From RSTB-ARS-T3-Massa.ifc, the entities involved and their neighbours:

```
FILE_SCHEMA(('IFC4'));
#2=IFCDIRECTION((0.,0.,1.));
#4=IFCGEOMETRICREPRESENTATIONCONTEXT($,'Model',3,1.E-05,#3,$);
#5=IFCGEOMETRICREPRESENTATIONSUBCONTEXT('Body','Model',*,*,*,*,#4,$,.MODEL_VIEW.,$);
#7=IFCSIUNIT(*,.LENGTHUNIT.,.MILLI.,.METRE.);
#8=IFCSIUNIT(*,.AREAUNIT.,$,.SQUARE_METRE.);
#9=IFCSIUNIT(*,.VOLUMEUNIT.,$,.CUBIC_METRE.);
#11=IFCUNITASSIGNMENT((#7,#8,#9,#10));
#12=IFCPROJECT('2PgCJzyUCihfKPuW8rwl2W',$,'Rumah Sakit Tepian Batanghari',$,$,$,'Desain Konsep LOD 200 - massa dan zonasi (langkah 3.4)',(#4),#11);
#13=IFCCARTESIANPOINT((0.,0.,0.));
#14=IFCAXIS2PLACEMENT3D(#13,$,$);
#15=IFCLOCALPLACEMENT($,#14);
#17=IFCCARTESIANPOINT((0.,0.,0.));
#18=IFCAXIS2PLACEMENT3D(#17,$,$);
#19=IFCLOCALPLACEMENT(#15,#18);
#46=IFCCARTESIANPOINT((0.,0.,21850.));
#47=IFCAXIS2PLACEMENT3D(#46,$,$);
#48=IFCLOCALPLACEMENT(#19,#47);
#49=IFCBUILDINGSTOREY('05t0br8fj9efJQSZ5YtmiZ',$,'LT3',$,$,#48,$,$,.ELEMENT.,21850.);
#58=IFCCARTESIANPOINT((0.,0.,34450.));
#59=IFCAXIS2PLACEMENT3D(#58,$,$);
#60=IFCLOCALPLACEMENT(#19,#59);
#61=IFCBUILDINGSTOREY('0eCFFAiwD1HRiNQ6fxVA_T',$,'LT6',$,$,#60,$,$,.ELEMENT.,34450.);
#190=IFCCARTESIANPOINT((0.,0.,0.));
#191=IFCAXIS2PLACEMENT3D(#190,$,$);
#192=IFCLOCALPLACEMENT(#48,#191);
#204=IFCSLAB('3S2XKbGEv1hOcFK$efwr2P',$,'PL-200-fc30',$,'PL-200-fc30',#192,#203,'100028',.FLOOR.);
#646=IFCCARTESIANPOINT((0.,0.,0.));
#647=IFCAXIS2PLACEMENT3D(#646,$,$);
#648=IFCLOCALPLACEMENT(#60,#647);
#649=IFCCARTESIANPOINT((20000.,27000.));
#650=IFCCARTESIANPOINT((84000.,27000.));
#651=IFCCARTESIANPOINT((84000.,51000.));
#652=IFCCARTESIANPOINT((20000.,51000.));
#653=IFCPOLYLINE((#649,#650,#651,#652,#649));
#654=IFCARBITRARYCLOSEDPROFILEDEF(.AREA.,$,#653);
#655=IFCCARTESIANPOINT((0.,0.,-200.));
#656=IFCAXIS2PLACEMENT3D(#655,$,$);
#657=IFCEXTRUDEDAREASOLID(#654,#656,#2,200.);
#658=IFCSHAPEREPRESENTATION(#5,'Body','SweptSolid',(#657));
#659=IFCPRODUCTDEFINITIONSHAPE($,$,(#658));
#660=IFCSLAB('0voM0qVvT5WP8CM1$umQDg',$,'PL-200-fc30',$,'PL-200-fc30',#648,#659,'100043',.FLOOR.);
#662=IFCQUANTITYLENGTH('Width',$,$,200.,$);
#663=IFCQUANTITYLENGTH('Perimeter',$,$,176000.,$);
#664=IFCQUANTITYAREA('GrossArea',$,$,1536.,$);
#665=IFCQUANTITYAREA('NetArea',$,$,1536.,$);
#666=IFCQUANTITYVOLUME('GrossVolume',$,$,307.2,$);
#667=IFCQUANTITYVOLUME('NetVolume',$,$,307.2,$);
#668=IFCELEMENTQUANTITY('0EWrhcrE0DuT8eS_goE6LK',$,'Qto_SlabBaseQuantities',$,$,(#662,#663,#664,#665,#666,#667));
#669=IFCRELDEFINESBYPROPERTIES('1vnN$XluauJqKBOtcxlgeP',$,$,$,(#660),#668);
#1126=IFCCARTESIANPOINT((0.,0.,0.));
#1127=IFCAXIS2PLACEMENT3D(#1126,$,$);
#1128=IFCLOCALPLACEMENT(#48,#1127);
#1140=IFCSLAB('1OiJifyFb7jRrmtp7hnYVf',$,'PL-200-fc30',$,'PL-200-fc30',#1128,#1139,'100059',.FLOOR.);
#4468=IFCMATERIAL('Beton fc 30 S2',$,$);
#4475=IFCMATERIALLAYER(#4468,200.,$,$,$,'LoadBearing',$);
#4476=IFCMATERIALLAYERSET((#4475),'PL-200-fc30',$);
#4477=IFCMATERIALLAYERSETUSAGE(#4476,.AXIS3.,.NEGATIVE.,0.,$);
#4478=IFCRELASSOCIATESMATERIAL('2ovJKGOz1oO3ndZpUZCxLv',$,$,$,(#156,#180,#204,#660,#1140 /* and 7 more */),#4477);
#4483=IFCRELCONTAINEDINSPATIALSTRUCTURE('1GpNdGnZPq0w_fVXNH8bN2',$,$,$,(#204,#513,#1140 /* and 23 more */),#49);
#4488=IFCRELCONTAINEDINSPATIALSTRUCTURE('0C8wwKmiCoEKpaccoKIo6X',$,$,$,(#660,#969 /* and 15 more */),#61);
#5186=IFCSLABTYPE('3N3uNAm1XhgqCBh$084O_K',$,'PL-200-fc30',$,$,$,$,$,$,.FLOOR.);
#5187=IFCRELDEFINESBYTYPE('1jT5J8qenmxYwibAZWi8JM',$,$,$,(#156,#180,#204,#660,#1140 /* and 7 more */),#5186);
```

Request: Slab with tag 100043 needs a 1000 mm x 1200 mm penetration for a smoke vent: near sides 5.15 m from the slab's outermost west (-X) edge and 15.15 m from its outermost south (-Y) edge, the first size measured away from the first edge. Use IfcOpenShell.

```python
import numpy as np
import ifcopenshell
import ifcopenshell.api.feature
import ifcopenshell.api.geometry
import ifcopenshell.api.pset
import ifcopenshell.api.root
import ifcopenshell.geom
import ifcopenshell.util.element
import ifcopenshell.util.placement
import ifcopenshell.util.representation
import ifcopenshell.util.shape
import ifcopenshell.util.unit

model = ifcopenshell.open("RSTB-ARS-T3-Massa.ifc")
unit_scale = ifcopenshell.util.unit.calculate_unit_scale(model)
area_scale = ifcopenshell.util.unit.calculate_unit_scale(model, "AREAUNIT")
volume_scale = ifcopenshell.util.unit.calculate_unit_scale(model, "VOLUMEUNIT")
settings = ifcopenshell.geom.settings()


def volume(element):
    """Net volume in cubic metres, openings subtracted."""
    shape = ifcopenshell.geom.create_shape(settings, element)
    return ifcopenshell.util.shape.get_volume(shape.geometry)


slab = model.by_guid("0voM0qVvT5WP8CM1$umQDg")
before = volume(slab)

# Extent in the slab's own axes, in metres. The edges named are its -X and -Y sides.
slab_shape = ifcopenshell.geom.create_shape(settings, slab)
vertices = ifcopenshell.util.shape.get_vertices(slab_shape.geometry)
x_min, y_min, bottom = vertices.min(axis=0)
top = vertices[:, 2].max()

opening = ifcopenshell.api.root.create_entity(model, ifc_class="IfcOpeningElement", name="Smoke vent opening", predefined_type="OPENING")
context = ifcopenshell.util.representation.get_context(model, "Model", "Body", "MODEL_VIEW")
width, depth = 1, 1.2
outline = [(0.0, 0.0), (width, 0.0), (width, depth), (0.0, depth), (0.0, 0.0)]
# Overshoot both faces by 50 mm so the cut is clean.
shape = ifcopenshell.api.geometry.add_slab_representation(
    model, context=context, depth=top - bottom + 0.1, polyline=outline
)
ifcopenshell.api.geometry.assign_representation(model, product=opening, representation=shape)

matrix = ifcopenshell.util.placement.get_local_placement(slab.ObjectPlacement)
matrix[:, 3] = matrix @ np.append(np.array([x_min + 5.15, y_min + 15.15, bottom - 0.05]) / unit_scale, 1.0)
ifcopenshell.api.geometry.edit_object_placement(model, product=opening, matrix=matrix, is_si=False)
ifcopenshell.api.feature.add_feature(model, feature=opening, element=slab)

after = volume(slab)

# Update the slab's stored quantities.
qto = model.by_id(ifcopenshell.util.element.get_pset(slab, "Qto_SlabBaseQuantities", should_inherit=False)["id"])
ifcopenshell.api.pset.edit_qto(model, qto=qto, properties={
    "NetArea": after / (top - bottom) / area_scale,
    "NetVolume": after / volume_scale,
})

print(f"slab volume {before:.3f} -> {after:.3f} m3")

model.write("RSTB-ARS-T3-Massa-out.ifc")
```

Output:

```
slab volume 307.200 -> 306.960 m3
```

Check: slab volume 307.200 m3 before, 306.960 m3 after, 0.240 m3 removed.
